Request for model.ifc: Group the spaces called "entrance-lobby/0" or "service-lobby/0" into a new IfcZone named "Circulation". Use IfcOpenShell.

First a look at what the model holds.

```python
import ifcopenshell

model = ifcopenshell.open("model.ifc")
print(model.schema)
seen = {}
for space in model.by_type("IfcSpace"):
    seen[space.Name] = seen.get(space.Name, 0) + 1
for name, count in sorted(seen.items(), key=str):
    print(count, "x", name)
print("zones:", [z.Name for z in model.by_type("IfcZone")][:20])
```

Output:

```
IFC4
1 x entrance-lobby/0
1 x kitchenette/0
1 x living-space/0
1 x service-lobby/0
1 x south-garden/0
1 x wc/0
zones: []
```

```python
import ifcopenshell
import ifcopenshell.api.group
import ifcopenshell.api.root

model = ifcopenshell.open("model.ifc")

names = {"entrance-lobby/0", "service-lobby/0"}
spaces = [s for s in model.by_type("IfcSpace") if s.Name in names]

zone = ifcopenshell.api.root.create_entity(model, ifc_class="IfcZone", name="Circulation")
ifcopenshell.api.group.assign_group(model, products=spaces, group=zone)
print(len(spaces), "spaces in", zone.Name)

model.write("model_v2.ifc")
```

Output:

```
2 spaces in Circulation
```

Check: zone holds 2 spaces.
